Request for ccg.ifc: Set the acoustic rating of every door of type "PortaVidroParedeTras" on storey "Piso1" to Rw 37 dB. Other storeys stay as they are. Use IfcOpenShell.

First a look at what the model holds.

```python
import ifcopenshell
import ifcopenshell.util.element

model = ifcopenshell.open("ccg.ifc")
print(model.schema)
storey = next(s for s in model.by_type("IfcBuildingStorey") if s.Name == "Piso1")
doors = [e for e in ifcopenshell.util.element.get_decomposition(storey) if e.is_a("IfcDoor")]
seen = {}
for e in doors:
    element_type = ifcopenshell.util.element.get_type(e)
    key = (element_type.Name if element_type != e and element_type else None, ifcopenshell.util.element.get_pset(e, "Pset_DoorCommon", "AcousticRating"))
    seen[key] = seen.get(key, 0) + 1
for (name, value), count in sorted(seen.items(), key=str):
    print(count, "x", name, "|", value)
```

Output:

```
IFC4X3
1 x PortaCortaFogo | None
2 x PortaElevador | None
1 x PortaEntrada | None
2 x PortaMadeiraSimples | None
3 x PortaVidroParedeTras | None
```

```python
import ifcopenshell
import ifcopenshell.api.pset
import ifcopenshell.util.element

model = ifcopenshell.open("ccg.ifc")

storey = next(s for s in model.by_type("IfcBuildingStorey") if s.Name == "Piso1")
doors = [e for e in ifcopenshell.util.element.get_decomposition(storey) if e.is_a("IfcDoor")]

count = 0
for e in doors:
    element_type = ifcopenshell.util.element.get_type(e)
    if element_type in (None, e) or element_type.Name != "PortaVidroParedeTras":
        continue
    # add_pset returns the element's existing set when there is one.
    pset = ifcopenshell.api.pset.add_pset(model, product=e, name="Pset_DoorCommon")
    ifcopenshell.api.pset.edit_pset(model, pset=pset, properties={"AcousticRating": "Rw 37 dB"})
    count += 1

print(count, "doors updated")

model.write("ccg_rev.ifc")
```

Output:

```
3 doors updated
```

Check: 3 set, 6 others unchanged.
